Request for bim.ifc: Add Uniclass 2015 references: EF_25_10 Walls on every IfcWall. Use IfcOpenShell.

First a look at what the model holds.

```python
import ifcopenshell

model = ifcopenshell.open("bim.ifc")
print(model.schema)
print("classifications:", [c.Name for c in model.by_type("IfcClassification")])
for ifc_class in ("IfcDoor", "IfcRoof", "IfcStair", "IfcWall", "IfcWindow"):
    print(ifc_class, len(model.by_type(ifc_class)))
```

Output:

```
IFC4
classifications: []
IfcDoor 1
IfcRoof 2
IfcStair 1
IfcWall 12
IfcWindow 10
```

```python
import ifcopenshell
import ifcopenshell.api.classification

model = ifcopenshell.open("bim.ifc")

system = ifcopenshell.api.classification.add_classification(model, classification="Uniclass 2015")

codes = {
    "IfcWall": ("EF_25_10", "Walls"),
}
for ifc_class, (code, name) in codes.items():
    products = model.by_type(ifc_class)
    ifcopenshell.api.classification.add_reference(
        model, products=products, classification=system, identification=code, name=name
    )
    print(code, len(products))

model.write("bim_edited.ifc")
```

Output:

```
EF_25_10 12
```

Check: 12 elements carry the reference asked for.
